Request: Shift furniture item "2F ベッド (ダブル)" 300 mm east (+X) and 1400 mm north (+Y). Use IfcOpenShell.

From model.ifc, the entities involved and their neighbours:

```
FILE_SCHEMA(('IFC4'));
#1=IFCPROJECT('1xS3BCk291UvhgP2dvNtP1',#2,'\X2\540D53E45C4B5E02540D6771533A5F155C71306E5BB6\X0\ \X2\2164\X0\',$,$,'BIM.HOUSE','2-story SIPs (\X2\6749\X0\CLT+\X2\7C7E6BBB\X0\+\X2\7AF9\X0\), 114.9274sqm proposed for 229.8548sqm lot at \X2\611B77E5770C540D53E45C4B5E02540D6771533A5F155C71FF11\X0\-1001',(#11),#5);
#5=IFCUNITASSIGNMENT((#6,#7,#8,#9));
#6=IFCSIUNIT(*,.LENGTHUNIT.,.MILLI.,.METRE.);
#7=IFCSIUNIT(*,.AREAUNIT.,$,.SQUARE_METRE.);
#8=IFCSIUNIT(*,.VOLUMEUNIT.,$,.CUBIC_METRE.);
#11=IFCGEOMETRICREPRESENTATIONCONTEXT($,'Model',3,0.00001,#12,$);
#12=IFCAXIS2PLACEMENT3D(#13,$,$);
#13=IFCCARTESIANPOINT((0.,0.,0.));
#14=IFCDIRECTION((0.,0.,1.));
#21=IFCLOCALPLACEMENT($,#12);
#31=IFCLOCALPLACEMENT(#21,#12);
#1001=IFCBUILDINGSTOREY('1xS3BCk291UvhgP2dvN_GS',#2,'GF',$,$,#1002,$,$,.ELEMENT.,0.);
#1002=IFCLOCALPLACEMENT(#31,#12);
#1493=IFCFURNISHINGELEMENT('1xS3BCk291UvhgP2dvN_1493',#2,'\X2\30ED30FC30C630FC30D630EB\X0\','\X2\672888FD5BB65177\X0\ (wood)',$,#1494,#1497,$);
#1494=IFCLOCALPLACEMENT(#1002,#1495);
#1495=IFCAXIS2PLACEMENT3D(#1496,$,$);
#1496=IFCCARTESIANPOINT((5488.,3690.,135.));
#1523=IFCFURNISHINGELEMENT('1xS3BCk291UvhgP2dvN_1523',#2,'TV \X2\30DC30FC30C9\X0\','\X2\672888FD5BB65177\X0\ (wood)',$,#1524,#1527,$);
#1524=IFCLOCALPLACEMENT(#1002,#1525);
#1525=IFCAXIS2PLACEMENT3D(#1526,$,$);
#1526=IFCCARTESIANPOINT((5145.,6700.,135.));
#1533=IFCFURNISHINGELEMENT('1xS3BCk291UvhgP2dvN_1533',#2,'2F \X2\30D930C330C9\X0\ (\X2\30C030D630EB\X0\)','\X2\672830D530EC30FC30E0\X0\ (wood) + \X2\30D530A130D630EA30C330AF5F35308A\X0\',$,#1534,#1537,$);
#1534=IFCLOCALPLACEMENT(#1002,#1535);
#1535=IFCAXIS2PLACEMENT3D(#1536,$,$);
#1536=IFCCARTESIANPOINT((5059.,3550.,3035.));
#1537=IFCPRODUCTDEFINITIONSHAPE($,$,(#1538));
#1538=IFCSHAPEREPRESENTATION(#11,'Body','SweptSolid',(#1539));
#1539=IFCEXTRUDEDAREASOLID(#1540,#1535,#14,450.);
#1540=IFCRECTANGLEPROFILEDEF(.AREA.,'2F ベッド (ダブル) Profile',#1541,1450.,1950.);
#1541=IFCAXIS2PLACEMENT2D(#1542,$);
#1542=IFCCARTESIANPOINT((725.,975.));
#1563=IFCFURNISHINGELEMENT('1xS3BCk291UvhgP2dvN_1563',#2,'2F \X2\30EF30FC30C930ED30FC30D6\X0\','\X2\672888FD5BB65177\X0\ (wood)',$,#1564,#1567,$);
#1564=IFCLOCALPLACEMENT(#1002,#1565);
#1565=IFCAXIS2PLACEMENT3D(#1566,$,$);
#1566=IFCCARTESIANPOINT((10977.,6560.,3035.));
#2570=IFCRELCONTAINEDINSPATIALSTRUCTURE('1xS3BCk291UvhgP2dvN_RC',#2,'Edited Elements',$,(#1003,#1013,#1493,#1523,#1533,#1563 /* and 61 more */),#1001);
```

```python
import ifcopenshell
import ifcopenshell.api.geometry
import ifcopenshell.util.placement

model = ifcopenshell.open("model.ifc")

item = model.by_guid("1xS3BCk291UvhgP2dvN_1533")
matrix = ifcopenshell.util.placement.get_local_placement(item.ObjectPlacement)
matrix[0, 3] += 300.0
matrix[1, 3] += 1400.0
ifcopenshell.api.geometry.edit_object_placement(model, product=item, matrix=matrix, is_si=False)

print(ifcopenshell.util.placement.get_local_placement(item.ObjectPlacement).round(3) + 0.0)

model.write("model_rev.ifc")
```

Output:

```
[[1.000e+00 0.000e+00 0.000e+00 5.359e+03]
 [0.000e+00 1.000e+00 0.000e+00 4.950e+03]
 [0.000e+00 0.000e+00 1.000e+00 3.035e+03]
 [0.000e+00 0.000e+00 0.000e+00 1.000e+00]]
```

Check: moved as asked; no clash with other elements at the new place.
